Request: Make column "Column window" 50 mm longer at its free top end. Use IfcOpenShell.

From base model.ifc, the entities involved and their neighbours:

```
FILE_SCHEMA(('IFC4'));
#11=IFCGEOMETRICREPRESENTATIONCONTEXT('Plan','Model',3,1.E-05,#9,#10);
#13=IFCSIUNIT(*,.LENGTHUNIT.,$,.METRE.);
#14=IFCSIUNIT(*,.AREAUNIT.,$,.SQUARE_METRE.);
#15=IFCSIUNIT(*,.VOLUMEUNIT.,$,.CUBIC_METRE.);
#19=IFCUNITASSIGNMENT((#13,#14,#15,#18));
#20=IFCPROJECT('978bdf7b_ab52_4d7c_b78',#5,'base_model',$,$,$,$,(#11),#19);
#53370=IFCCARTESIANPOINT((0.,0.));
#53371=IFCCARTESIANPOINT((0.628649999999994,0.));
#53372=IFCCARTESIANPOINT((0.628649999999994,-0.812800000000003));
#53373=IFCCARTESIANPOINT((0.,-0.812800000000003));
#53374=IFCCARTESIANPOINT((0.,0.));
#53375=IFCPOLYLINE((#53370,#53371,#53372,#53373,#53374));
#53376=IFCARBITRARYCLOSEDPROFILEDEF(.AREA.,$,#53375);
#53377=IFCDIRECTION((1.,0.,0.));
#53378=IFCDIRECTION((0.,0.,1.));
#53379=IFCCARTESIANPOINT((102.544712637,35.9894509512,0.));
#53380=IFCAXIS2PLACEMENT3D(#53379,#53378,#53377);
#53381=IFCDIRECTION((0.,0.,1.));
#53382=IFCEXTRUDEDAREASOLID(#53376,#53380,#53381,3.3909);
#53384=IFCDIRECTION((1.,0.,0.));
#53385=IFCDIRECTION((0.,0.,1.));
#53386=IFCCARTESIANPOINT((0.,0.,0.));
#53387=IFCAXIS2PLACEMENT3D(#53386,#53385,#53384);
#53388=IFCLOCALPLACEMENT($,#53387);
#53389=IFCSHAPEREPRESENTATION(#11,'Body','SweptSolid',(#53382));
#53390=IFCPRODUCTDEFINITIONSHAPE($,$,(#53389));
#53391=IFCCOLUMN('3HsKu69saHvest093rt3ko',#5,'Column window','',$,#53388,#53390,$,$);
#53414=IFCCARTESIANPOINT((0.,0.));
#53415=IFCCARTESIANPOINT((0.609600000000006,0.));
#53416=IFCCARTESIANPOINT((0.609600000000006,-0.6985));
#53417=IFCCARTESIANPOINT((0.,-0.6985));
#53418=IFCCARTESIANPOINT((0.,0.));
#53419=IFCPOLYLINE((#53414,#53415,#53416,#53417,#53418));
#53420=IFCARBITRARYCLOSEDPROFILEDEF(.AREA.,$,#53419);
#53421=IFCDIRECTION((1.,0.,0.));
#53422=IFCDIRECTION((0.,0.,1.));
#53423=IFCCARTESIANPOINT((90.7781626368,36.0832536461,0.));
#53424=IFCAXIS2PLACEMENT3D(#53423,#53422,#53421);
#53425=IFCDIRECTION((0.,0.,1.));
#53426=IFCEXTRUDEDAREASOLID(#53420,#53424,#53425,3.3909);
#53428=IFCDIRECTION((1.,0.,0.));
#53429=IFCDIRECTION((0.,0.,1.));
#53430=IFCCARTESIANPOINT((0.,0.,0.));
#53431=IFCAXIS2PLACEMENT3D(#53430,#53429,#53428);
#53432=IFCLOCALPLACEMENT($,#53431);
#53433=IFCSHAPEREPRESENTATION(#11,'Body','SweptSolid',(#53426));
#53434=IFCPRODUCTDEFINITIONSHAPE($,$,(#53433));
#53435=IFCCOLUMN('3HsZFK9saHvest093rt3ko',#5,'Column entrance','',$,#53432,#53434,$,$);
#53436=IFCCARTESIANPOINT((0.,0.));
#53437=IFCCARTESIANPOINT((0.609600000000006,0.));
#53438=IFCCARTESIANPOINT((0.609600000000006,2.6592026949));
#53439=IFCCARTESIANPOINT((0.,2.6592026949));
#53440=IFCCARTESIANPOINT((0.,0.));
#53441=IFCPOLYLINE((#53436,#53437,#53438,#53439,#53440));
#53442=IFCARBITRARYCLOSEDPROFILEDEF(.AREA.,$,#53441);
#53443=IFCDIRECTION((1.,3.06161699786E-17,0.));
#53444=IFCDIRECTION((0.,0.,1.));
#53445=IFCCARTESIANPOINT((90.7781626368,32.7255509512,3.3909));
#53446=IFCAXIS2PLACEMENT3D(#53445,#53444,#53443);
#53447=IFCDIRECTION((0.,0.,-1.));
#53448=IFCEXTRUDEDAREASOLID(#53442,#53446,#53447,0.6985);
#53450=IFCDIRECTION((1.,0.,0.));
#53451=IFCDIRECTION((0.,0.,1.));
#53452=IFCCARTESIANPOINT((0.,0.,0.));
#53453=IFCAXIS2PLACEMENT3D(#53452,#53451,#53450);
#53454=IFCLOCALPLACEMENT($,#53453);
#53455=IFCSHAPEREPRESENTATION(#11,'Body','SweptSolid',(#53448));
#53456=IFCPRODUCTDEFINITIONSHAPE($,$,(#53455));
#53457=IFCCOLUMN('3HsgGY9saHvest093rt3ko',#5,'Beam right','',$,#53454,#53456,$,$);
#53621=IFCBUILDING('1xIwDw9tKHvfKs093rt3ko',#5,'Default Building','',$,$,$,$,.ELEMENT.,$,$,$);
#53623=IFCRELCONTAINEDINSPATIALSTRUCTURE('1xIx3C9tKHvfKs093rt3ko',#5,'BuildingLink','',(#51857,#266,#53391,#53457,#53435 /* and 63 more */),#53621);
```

```python
import ifcopenshell
import ifcopenshell.util.unit

model = ifcopenshell.open("base model.ifc")
unit_scale = ifcopenshell.util.unit.calculate_unit_scale(model)

member = model.by_guid("3HsKu69saHvest093rt3ko")
change = 0.05 / unit_scale

# The extrusion runs towards the end named, so only its depth changes.
body = next(r for r in member.Representation.Representations if r.RepresentationIdentifier == "Body")
solid = body.Items[0]
old_length = solid.Depth
solid.Depth += change

print(f"length {old_length:g} -> {solid.Depth:g}")

model.write("base model_rev.ifc")
```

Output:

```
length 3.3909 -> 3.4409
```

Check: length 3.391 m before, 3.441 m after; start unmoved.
